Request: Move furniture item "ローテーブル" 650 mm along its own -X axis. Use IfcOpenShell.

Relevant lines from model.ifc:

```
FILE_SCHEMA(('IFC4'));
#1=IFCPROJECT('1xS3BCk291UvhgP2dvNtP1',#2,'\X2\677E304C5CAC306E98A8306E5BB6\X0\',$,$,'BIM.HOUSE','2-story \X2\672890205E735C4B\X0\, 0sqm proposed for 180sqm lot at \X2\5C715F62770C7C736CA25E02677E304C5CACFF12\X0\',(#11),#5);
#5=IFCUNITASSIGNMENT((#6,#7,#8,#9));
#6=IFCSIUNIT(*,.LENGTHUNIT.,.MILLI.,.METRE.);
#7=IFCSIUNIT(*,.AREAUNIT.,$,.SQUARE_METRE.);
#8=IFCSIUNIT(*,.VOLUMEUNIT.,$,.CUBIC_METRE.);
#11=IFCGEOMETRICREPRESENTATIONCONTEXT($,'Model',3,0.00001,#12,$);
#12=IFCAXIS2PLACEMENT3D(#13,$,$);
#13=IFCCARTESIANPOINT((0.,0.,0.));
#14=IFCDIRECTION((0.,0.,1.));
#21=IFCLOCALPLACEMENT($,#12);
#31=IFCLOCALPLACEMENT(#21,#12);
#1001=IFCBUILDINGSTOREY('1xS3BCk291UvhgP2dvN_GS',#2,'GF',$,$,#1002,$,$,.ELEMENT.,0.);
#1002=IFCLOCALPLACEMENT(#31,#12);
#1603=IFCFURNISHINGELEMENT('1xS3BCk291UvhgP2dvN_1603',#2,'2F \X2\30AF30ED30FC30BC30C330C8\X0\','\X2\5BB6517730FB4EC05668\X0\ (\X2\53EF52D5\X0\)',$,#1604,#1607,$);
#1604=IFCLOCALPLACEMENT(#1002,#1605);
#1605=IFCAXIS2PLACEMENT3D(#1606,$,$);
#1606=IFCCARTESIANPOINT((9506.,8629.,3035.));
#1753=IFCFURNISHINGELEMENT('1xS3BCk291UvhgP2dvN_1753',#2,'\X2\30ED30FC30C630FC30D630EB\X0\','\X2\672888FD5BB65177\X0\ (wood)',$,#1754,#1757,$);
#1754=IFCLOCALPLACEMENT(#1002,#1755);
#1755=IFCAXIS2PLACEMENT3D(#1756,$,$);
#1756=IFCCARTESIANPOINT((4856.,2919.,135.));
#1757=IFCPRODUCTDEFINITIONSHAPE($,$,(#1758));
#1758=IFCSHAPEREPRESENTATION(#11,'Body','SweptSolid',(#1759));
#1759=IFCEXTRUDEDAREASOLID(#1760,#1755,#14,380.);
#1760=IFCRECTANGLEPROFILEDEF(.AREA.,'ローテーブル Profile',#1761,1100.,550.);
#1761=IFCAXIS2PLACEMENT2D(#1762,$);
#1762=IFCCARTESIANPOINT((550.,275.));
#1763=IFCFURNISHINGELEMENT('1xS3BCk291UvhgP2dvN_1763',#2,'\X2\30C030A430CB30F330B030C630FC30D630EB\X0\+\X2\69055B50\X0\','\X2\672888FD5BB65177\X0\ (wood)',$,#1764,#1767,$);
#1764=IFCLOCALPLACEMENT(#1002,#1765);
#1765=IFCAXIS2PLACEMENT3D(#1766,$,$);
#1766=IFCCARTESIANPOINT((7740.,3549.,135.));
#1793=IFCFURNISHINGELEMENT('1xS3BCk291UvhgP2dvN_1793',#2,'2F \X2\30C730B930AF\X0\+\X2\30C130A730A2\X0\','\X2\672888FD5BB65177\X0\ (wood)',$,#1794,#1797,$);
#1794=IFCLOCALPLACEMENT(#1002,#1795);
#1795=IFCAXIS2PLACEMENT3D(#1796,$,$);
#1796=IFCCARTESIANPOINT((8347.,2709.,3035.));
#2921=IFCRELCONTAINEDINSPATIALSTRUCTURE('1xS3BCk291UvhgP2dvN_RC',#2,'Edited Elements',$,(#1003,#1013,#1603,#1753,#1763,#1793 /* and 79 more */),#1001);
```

```python
import ifcopenshell
import ifcopenshell.api.geometry
import ifcopenshell.util.placement
import ifcopenshell.util.unit

model = ifcopenshell.open("model.ifc")
unit_scale = ifcopenshell.util.unit.calculate_unit_scale(model)

item = model.by_id(1753)
matrix = ifcopenshell.util.placement.get_local_placement(item.ObjectPlacement)
matrix[:3, 3] -= matrix[:3, 0] * 0.65 / unit_scale
ifcopenshell.api.geometry.edit_object_placement(model, product=item, matrix=matrix, is_si=False)

print(ifcopenshell.util.placement.get_local_placement(item.ObjectPlacement).round(3) + 0.0)

model.write("model-out.ifc")
```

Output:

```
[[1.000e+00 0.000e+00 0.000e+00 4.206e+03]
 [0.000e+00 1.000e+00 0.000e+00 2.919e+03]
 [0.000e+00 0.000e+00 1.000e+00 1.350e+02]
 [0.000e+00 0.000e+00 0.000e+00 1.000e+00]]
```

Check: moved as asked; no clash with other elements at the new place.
